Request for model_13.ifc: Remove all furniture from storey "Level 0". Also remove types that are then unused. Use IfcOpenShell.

First a look at what the model holds.

```python
import ifcopenshell
import ifcopenshell.util.element

model = ifcopenshell.open("model_13.ifc")
print(model.schema)
storey = next(s for s in model.by_type("IfcBuildingStorey") if s.Name == "Level 0")
furniture = [e for e in ifcopenshell.util.element.get_decomposition(storey) if e.is_a("IfcFurnishingElement")]
seen = {}
for e in furniture:
    element_type = ifcopenshell.util.element.get_type(e)
    name = element_type.Name if element_type not in (None, e) else None
    seen[name] = seen.get(name, 0) + 1
for name, count in sorted(seen.items(), key=str):
    print(count, "x", name)
```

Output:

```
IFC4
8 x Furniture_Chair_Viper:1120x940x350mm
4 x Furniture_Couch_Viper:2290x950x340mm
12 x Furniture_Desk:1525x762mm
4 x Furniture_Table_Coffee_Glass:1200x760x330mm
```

```python
import ifcopenshell
import ifcopenshell.api.root
import ifcopenshell.util.element

model = ifcopenshell.open("model_13.ifc")

storey = next(s for s in model.by_type("IfcBuildingStorey") if s.Name == "Level 0")
furniture = [e for e in ifcopenshell.util.element.get_decomposition(storey) if e.is_a("IfcFurnishingElement")]
types = {ifcopenshell.util.element.get_type(e) for e in furniture} - {None, *furniture}

for e in furniture:
    ifcopenshell.api.root.remove_product(model, product=e)
print(len(furniture), "removed")

unused = [t for t in types if not ifcopenshell.util.element.get_types(t)]
for t in unused:
    ifcopenshell.api.root.remove_product(model, product=t)
print(len(unused), "unused types removed")

model.write("model_13_rev.ifc")
```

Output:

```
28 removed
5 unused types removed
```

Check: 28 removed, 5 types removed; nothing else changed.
